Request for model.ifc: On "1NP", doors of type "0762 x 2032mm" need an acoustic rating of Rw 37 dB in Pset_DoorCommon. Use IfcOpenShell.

First a look at what the model holds.

```python
import ifcopenshell
import ifcopenshell.util.element

model = ifcopenshell.open("model.ifc")
print(model.schema)
storey = next(s for s in model.by_type("IfcBuildingStorey") if s.Name == "1NP")
doors = [e for e in ifcopenshell.util.element.get_decomposition(storey) if e.is_a("IfcDoor")]
seen = {}
for e in doors:
    element_type = ifcopenshell.util.element.get_type(e)
    key = (element_type.Name if element_type != e and element_type else None, ifcopenshell.util.element.get_pset(e, "Pset_DoorCommon", "AcousticRating"))
    seen[key] = seen.get(key, 0) + 1
for (name, value), count in sorted(seen.items(), key=str):
    print(count, "x", name, "|", value)
```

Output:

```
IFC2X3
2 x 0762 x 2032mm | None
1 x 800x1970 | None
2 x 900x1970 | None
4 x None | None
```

```python
import ifcopenshell
import ifcopenshell.api.pset
import ifcopenshell.util.element

model = ifcopenshell.open("model.ifc")

storey = next(s for s in model.by_type("IfcBuildingStorey") if s.Name == "1NP")
doors = [e for e in ifcopenshell.util.element.get_decomposition(storey) if e.is_a("IfcDoor")]

count = 0
for e in doors:
    element_type = ifcopenshell.util.element.get_type(e)
    if element_type in (None, e) or element_type.Name != "0762 x 2032mm":
        continue
    # add_pset returns the element's existing set when there is one.
    pset = ifcopenshell.api.pset.add_pset(model, product=e, name="Pset_DoorCommon")
    ifcopenshell.api.pset.edit_pset(model, pset=pset, properties={"AcousticRating": "Rw 37 dB"})
    count += 1

print(count, "doors updated")

model.write("model_edited.ifc")
```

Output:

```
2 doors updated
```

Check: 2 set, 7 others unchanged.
